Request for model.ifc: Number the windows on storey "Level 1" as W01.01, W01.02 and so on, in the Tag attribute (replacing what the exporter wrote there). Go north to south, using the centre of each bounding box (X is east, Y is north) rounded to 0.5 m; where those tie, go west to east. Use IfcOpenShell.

First a look at what the model holds.

```python
import ifcopenshell
import ifcopenshell.util.element
import ifcopenshell.util.placement

model = ifcopenshell.open("model.ifc")
print(model.schema)
storey = next(s for s in model.by_type("IfcBuildingStorey") if s.Name == "Level 1")
windows = [e for e in ifcopenshell.util.element.get_decomposition(storey) if e.is_a("IfcWindow")]
for e in sorted(windows, key=lambda e: e.id()):
    origin = ifcopenshell.util.placement.get_local_placement(e.ObjectPlacement)[:3, 3]
    print(e.id(), e.Tag, e.Name, origin.round(2) + 0.0, sep=" | ")
```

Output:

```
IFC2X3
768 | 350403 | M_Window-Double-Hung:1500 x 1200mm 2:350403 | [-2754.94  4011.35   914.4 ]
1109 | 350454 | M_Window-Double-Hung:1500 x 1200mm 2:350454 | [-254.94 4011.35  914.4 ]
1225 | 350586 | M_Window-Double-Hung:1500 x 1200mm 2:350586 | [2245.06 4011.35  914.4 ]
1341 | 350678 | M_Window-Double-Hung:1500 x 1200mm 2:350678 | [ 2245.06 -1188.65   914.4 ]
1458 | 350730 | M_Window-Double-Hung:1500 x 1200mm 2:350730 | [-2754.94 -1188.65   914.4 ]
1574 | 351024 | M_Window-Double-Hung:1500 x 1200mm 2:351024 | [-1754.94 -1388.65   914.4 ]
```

```python
import ifcopenshell
import ifcopenshell.geom
import ifcopenshell.util.element
import ifcopenshell.util.shape

model = ifcopenshell.open("model.ifc")
settings = ifcopenshell.geom.settings()
settings.set("use-world-coords", True)


def centre(element):
    shape = ifcopenshell.geom.create_shape(settings, element)
    return ifcopenshell.util.shape.get_bbox_centroid(shape.geometry)


storey = next(s for s in model.by_type("IfcBuildingStorey") if s.Name == "Level 1")
windows = [e for e in ifcopenshell.util.element.get_decomposition(storey) if e.is_a("IfcWindow")]

# Insertion points can sit at a corner or the storey origin, so sort by the geometry (in metres).
centres = {e: centre(e) for e in windows}
windows.sort(key=lambda e: (-round(centres[e][1] / 0.5), centres[e][0]))

for i, e in enumerate(windows, start=1):
    number = f"W01.{i:02d}"
    e.Tag = number
    print(e.id(), number)

model.write("model-out.ifc")
```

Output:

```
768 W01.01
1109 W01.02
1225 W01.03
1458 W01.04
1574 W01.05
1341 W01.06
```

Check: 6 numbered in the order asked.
